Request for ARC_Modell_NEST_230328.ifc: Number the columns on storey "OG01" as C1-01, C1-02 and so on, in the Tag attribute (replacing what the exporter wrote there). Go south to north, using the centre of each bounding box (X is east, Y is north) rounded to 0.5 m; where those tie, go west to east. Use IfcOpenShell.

First a look at what the model holds.

```python
import ifcopenshell
import ifcopenshell.util.element
import ifcopenshell.util.placement

model = ifcopenshell.open("ARC_Modell_NEST_230328.ifc")
print(model.schema)
storey = next(s for s in model.by_type("IfcBuildingStorey") if s.Name == "OG01")
columns = [e for e in ifcopenshell.util.element.get_decomposition(storey) if e.is_a("IfcColumn")]
for e in sorted(columns, key=lambda e: e.id()):
    origin = ifcopenshell.util.placement.get_local_placement(e.ObjectPlacement)[:3, 3]
    print(e.id(), e.Tag, e.Name, origin.round(2) + 0.0, sep=" | ")
```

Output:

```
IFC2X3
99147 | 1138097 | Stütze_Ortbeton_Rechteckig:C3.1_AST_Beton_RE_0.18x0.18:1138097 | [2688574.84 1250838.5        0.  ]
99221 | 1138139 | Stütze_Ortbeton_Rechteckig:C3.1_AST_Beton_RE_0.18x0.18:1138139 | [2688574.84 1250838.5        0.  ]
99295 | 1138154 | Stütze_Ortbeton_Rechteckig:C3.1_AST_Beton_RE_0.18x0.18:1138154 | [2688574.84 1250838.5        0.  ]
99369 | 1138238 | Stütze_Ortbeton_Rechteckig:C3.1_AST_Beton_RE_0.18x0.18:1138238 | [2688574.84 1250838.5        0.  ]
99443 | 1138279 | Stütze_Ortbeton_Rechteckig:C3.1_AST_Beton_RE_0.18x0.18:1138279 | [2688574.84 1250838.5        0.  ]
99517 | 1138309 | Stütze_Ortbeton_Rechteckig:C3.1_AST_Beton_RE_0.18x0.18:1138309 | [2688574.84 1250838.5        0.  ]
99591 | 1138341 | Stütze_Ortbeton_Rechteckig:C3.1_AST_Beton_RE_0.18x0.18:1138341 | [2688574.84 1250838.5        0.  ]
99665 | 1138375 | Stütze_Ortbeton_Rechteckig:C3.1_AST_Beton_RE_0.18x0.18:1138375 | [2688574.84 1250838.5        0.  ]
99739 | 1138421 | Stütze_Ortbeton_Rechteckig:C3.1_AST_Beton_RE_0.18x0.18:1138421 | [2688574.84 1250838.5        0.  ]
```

```python
import ifcopenshell
import ifcopenshell.geom
import ifcopenshell.util.element
import ifcopenshell.util.shape

model = ifcopenshell.open("ARC_Modell_NEST_230328.ifc")
settings = ifcopenshell.geom.settings()
settings.set("use-world-coords", True)


def centre(element):
    shape = ifcopenshell.geom.create_shape(settings, element)
    return ifcopenshell.util.shape.get_bbox_centroid(shape.geometry)


storey = next(s for s in model.by_type("IfcBuildingStorey") if s.Name == "OG01")
columns = [e for e in ifcopenshell.util.element.get_decomposition(storey) if e.is_a("IfcColumn")]

# Insertion points can sit at a corner or the storey origin, so sort by the geometry (in metres).
centres = {e: centre(e) for e in columns}
columns.sort(key=lambda e: (round(centres[e][1] / 0.5), centres[e][0]))

for i, e in enumerate(columns, start=1):
    number = f"C1-{i:02d}"
    e.Tag = number
    print(e.id(), number)

model.write("ARC_Modell_NEST_230328_updated.ifc")
```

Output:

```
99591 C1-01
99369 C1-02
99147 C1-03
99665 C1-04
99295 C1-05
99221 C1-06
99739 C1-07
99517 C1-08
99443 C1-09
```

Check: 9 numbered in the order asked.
